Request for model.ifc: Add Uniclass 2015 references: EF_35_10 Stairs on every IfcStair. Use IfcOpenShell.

First a look at what the model holds.

```python
import ifcopenshell

model = ifcopenshell.open("model.ifc")
print(model.schema)
print("classifications:", [c.Name for c in model.by_type("IfcClassification")])
for ifc_class in ("IfcDoor", "IfcRoof", "IfcStair", "IfcWall", "IfcWindow"):
    print(ifc_class, len(model.by_type(ifc_class)))
```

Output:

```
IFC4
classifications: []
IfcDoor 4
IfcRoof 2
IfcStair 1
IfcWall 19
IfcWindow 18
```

```python
import ifcopenshell
import ifcopenshell.api.classification

model = ifcopenshell.open("model.ifc")

system = ifcopenshell.api.classification.add_classification(model, classification="Uniclass 2015")

codes = {
    "IfcStair": ("EF_35_10", "Stairs"),
}
for ifc_class, (code, name) in codes.items():
    products = model.by_type(ifc_class)
    ifcopenshell.api.classification.add_reference(
        model, products=products, classification=system, identification=code, name=name
    )
    print(code, len(products))

model.write("model-out.ifc")
```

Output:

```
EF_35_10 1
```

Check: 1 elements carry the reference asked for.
